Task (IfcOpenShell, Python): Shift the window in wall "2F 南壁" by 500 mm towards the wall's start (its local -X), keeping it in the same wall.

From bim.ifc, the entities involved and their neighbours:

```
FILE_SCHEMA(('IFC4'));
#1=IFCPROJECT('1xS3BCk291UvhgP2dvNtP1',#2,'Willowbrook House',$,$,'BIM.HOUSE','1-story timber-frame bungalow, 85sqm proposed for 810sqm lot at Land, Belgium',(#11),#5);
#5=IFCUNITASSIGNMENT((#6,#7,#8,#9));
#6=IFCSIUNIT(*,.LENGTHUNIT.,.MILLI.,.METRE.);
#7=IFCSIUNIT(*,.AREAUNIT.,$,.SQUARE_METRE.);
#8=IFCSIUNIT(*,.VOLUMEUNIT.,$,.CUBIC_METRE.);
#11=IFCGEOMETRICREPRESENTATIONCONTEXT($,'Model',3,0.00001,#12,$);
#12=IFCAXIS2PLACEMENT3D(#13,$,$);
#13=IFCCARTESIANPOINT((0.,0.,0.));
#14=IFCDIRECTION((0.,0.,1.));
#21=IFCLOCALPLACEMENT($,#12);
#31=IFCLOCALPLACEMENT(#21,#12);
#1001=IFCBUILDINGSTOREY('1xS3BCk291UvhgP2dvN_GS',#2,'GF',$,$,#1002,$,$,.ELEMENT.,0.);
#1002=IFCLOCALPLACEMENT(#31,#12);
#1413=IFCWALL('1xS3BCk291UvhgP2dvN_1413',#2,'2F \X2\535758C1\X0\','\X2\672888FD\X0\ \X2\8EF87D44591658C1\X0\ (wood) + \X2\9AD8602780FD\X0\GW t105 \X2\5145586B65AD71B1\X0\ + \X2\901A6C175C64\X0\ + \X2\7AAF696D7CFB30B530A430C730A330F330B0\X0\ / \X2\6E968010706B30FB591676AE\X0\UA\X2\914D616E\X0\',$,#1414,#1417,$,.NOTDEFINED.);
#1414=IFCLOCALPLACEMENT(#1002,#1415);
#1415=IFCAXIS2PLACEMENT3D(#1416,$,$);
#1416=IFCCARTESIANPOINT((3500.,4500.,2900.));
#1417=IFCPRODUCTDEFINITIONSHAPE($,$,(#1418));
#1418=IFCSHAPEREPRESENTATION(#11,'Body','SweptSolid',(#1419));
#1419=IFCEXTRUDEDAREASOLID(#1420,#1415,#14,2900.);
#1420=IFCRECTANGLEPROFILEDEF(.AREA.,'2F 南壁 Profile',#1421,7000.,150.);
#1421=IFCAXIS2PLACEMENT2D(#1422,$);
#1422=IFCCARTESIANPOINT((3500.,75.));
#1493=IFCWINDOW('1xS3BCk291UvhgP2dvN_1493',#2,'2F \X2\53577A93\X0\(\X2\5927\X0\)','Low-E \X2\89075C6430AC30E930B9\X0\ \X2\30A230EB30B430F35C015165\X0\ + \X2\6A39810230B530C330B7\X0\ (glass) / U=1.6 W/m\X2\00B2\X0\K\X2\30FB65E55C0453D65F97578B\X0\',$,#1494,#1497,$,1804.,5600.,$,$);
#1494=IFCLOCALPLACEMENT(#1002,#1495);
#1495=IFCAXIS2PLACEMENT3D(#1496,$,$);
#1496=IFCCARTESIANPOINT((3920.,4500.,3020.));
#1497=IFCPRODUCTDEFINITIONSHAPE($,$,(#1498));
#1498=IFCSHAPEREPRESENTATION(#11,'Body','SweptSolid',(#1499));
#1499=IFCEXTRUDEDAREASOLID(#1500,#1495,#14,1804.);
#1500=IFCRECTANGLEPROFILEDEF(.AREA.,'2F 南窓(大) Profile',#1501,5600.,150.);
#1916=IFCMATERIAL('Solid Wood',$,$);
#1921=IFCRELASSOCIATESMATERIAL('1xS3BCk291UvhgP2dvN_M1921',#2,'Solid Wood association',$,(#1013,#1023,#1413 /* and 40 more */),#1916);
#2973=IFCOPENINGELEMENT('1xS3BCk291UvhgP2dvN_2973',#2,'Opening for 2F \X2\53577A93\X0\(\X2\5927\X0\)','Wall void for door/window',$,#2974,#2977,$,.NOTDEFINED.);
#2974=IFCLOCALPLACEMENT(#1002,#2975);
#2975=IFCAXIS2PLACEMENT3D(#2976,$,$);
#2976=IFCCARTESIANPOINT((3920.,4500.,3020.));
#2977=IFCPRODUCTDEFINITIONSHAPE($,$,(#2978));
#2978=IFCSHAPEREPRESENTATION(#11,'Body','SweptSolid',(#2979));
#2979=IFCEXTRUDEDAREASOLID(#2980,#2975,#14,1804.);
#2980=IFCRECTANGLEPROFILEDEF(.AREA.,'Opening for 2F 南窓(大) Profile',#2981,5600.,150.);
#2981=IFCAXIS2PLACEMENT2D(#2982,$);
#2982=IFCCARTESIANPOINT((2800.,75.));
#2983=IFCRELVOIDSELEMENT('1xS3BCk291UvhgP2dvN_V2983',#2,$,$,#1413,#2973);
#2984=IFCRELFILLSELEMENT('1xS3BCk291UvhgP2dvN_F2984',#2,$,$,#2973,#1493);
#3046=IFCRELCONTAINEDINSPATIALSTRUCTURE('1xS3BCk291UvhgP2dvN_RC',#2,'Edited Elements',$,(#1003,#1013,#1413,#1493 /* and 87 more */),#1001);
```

```python
import ifcopenshell
import ifcopenshell.api.geometry
import ifcopenshell.util.placement
import ifcopenshell.util.unit

model = ifcopenshell.open("bim.ifc")
unit_scale = ifcopenshell.util.unit.calculate_unit_scale(model)

window = model.by_guid("1xS3BCk291UvhgP2dvN_1493")
opening = window.FillsVoids[0].RelatingOpeningElement
wall = opening.VoidsElements[0].RelatingBuildingElement

wall_matrix = ifcopenshell.util.placement.get_local_placement(wall.ObjectPlacement)
shift = wall_matrix[:3, 0] * -0.5 / unit_scale
before = ifcopenshell.util.placement.get_local_placement(window.ObjectPlacement)[:3, 3].copy()

# The window is not placed relative to its opening, so move both.
for product in (opening, window):
    matrix = ifcopenshell.util.placement.get_local_placement(product.ObjectPlacement)
    matrix[:3, 3] += shift
    ifcopenshell.api.geometry.edit_object_placement(model, product=product, matrix=matrix, is_si=False)

after = ifcopenshell.util.placement.get_local_placement(window.ObjectPlacement)[:3, 3]
print("window moved by", (after - before).round(3) + 0.0)

model.write("bim_v2.ifc")
```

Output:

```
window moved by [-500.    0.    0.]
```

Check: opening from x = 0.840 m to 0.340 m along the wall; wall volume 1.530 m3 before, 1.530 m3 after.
